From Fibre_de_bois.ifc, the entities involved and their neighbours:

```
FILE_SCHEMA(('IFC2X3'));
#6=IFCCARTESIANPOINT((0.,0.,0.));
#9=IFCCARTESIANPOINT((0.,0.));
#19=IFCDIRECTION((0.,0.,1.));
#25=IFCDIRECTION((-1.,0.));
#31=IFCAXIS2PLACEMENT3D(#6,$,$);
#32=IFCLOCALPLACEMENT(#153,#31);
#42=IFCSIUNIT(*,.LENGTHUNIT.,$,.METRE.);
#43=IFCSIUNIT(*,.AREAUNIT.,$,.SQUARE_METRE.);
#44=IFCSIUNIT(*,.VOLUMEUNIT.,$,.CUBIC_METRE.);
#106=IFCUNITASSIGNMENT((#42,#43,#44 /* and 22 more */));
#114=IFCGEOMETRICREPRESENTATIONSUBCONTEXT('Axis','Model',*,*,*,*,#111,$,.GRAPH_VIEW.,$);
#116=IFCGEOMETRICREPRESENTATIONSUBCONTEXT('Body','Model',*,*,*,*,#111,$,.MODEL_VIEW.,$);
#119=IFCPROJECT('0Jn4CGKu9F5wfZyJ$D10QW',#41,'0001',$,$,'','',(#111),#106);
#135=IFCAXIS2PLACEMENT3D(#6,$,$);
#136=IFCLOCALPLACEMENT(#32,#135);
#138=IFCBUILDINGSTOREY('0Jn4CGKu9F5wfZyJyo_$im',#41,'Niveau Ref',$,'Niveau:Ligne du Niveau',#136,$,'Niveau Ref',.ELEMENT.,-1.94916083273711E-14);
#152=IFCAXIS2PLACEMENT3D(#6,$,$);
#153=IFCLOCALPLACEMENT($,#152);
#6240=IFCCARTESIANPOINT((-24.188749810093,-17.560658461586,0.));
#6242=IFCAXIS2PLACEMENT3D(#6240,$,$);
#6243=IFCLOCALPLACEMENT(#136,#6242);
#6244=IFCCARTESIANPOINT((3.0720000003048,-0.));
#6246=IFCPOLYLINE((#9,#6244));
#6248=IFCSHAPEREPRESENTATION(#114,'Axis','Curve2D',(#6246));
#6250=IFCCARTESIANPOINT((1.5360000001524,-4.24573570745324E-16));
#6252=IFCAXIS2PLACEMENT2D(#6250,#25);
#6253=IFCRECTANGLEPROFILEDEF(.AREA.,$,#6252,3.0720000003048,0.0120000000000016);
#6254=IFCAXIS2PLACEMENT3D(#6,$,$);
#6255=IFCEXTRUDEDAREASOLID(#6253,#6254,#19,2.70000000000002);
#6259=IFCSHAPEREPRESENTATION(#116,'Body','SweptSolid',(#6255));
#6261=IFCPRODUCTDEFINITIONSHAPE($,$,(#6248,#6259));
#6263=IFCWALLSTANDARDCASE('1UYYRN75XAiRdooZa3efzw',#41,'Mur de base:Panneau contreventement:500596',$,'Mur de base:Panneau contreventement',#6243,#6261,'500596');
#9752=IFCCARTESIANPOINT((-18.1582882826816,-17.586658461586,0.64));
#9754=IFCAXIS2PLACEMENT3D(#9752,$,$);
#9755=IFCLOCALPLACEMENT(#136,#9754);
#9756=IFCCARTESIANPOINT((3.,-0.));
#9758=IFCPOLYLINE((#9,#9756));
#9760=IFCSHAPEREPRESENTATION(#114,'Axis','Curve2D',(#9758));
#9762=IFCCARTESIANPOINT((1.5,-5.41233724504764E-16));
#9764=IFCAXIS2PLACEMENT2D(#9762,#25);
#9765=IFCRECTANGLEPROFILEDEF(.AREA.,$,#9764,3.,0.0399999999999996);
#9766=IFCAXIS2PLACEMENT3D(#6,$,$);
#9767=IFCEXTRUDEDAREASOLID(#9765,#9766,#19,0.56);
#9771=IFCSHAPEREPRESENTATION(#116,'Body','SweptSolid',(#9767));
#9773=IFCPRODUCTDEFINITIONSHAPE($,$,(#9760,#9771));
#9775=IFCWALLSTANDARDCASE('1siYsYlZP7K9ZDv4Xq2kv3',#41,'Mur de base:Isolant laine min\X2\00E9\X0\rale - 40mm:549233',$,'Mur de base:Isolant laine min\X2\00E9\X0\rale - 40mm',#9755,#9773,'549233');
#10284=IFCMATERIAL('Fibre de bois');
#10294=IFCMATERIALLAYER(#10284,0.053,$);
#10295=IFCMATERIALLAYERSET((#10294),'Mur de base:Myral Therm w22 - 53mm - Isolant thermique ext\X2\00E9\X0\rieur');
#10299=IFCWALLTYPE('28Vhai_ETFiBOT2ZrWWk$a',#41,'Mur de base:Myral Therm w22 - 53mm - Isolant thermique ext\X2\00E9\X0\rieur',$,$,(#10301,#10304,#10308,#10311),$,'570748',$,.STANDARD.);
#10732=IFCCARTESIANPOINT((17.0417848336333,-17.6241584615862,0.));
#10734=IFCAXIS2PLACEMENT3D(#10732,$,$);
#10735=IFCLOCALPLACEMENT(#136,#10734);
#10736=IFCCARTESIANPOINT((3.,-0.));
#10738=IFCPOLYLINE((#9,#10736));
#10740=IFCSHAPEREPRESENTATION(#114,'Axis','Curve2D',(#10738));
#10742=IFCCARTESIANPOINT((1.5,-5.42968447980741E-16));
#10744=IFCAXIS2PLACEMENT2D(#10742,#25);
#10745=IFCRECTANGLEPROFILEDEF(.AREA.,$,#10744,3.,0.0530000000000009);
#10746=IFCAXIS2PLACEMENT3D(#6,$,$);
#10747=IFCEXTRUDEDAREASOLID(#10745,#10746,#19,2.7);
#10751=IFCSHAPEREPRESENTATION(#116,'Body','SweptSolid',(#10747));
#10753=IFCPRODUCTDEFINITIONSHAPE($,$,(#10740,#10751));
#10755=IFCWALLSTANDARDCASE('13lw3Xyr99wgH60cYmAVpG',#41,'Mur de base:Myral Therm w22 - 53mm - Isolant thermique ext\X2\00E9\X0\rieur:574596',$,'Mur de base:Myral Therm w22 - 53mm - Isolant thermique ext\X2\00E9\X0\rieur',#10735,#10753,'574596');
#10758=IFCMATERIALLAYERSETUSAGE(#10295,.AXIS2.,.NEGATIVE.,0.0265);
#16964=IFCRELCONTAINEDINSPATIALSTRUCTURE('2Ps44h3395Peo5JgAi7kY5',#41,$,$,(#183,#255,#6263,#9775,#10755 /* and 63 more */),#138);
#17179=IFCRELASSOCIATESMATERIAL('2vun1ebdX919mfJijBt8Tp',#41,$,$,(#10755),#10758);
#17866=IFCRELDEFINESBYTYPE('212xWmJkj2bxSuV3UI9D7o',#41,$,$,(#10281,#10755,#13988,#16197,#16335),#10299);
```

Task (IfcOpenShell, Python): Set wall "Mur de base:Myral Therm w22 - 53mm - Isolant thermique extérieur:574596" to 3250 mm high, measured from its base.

```python
import ifcopenshell
import ifcopenshell.geom
import ifcopenshell.util.representation
import ifcopenshell.util.shape
import ifcopenshell.util.unit

model = ifcopenshell.open("Fibre_de_bois.ifc")
unit_scale = ifcopenshell.util.unit.calculate_unit_scale(model)
settings = ifcopenshell.geom.settings()


def volume(element):
    """Net volume in cubic metres, openings subtracted."""
    shape = ifcopenshell.geom.create_shape(settings, element)
    return ifcopenshell.util.shape.get_volume(shape.geometry)


wall = model.by_guid("13lw3Xyr99wgH60cYmAVpG")
before = volume(wall)

body = ifcopenshell.util.representation.get_representation(wall, "Model", "Body")
solid = body.Items[0]
old_height = solid.Depth
solid.Depth = 3.25 / unit_scale
after = volume(wall)

print(f"height {old_height:g} -> {solid.Depth:g}, volume {before:.3f} -> {after:.3f} m3")

model.write("Fibre_de_bois_rev.ifc")
```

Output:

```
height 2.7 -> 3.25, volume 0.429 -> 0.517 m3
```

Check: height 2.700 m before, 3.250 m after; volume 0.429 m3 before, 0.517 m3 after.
